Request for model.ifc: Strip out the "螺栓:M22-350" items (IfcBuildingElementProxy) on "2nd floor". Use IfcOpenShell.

First a look at what the model holds.

```python
import ifcopenshell
import ifcopenshell.util.element

model = ifcopenshell.open("model.ifc")
print(model.schema)
storey = next(s for s in model.by_type("IfcBuildingStorey") if s.Name == "2nd floor")
proxies = [e for e in ifcopenshell.util.element.get_decomposition(storey) if e.is_a("IfcBuildingElementProxy")]
seen = {}
for e in proxies:
    element_type = ifcopenshell.util.element.get_type(e)
    name = element_type.Name if element_type not in (None, e) else None
    seen[name] = seen.get(name, 0) + 1
for name, count in sorted(seen.items(), key=str):
    print(count, "x", name)
```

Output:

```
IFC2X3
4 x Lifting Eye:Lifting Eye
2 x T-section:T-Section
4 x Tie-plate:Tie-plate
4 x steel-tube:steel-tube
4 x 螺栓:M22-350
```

```python
import ifcopenshell
import ifcopenshell.api.root
import ifcopenshell.util.element

model = ifcopenshell.open("model.ifc")

storey = next(s for s in model.by_type("IfcBuildingStorey") if s.Name == "2nd floor")
proxies = [e for e in ifcopenshell.util.element.get_decomposition(storey) if e.is_a("IfcBuildingElementProxy")]
targets = [e for e in proxies if (t := ifcopenshell.util.element.get_type(e)) not in (None, e) and t.Name == "螺栓:M22-350"]

for e in targets:
    ifcopenshell.api.root.remove_product(model, product=e)
print(len(targets), "removed")

model.write("model_rev.ifc")
```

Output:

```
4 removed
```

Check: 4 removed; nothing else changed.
